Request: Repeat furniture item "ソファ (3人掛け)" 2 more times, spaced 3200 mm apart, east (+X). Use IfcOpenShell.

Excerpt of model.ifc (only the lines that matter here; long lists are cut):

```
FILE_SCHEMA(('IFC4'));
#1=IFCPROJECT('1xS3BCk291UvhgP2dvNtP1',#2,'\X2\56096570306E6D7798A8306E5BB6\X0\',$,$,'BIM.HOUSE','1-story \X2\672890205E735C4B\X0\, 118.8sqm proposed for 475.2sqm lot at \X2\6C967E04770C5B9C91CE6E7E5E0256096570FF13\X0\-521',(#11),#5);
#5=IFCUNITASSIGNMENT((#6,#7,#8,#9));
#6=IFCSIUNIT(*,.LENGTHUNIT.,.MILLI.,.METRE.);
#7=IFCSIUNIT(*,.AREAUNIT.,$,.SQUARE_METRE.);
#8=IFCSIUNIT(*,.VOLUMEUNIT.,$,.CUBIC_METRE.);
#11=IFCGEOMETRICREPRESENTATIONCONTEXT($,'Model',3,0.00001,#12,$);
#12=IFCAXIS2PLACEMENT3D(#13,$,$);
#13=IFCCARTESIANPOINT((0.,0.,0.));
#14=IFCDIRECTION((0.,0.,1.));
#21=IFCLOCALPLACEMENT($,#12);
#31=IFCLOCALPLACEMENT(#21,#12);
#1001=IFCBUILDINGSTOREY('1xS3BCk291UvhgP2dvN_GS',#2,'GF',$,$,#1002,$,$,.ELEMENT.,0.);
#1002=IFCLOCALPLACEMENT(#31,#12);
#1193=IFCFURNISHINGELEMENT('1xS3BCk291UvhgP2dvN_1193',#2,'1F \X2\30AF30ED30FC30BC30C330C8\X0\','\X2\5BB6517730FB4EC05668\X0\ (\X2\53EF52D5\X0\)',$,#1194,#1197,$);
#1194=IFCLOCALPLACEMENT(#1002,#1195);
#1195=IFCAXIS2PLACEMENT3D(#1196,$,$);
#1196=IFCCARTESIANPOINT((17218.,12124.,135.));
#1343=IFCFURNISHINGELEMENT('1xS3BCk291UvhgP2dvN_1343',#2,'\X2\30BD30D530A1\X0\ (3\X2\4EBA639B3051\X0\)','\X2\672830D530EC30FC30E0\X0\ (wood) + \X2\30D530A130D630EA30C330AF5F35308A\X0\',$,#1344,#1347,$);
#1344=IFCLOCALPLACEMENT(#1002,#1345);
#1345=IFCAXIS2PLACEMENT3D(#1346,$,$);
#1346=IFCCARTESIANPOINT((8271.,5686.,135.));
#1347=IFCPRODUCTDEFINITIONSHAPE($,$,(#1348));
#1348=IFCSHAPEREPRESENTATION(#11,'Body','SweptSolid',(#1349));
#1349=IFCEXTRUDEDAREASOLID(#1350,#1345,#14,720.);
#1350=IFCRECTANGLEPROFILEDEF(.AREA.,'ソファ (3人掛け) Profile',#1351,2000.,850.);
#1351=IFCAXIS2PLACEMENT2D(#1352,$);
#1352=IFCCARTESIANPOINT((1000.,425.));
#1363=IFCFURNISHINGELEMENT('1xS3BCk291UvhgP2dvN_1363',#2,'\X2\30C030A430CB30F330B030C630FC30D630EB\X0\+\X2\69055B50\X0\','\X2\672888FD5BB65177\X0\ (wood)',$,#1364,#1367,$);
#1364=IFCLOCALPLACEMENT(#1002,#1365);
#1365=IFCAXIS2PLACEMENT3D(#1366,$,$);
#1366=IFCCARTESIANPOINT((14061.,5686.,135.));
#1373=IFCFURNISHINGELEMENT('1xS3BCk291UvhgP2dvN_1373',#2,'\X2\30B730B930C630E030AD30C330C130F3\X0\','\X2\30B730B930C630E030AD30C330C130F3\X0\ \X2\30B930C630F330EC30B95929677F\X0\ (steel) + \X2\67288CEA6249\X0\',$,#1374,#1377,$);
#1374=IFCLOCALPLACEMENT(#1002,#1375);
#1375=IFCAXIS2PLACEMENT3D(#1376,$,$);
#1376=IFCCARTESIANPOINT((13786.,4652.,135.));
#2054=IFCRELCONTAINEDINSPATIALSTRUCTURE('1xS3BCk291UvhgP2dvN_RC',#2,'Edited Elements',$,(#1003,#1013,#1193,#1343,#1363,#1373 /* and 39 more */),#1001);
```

```python
import numpy as np
import ifcopenshell
import ifcopenshell.api.geometry
import ifcopenshell.api.root
import ifcopenshell.util.element
import ifcopenshell.util.placement
import ifcopenshell.util.unit

model = ifcopenshell.open("model.ifc")
unit_scale = ifcopenshell.util.unit.calculate_unit_scale(model)


def reuse_history(source, copy):
    """copy_class also copies each property set's owner history, people and application; keep the originals."""
    for rel in copy.IsDefinedBy:
        if rel.is_a("IfcRelDefinesByProperties") and (history := rel.RelatingPropertyDefinition.OwnerHistory):
            rel.RelatingPropertyDefinition.OwnerHistory = source.OwnerHistory
            ifcopenshell.util.element.remove_deep2(model, history)


source = model.by_guid("1xS3BCk291UvhgP2dvN_1343")
base = ifcopenshell.util.placement.get_local_placement(source.ObjectPlacement)
step = np.array([1.0, 0.0, 0.0]) * 3.2 / unit_scale

for i in range(1, 3):
    copy = ifcopenshell.api.root.copy_class(model, product=source)
    copy.Representation = ifcopenshell.util.element.copy_deep(
        model, source.Representation, exclude=["IfcGeometricRepresentationContext", "IfcRepresentationMap"]
    )
    reuse_history(source, copy)
    matrix = base.copy()
    matrix[:3, 3] += i * step
    print("added at", matrix[:3, 3].round(3) + 0.0)
    ifcopenshell.api.geometry.edit_object_placement(model, product=copy, matrix=matrix, is_si=False)

model.write("model_rev.ifc")
```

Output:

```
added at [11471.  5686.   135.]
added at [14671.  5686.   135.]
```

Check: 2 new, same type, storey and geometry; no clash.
